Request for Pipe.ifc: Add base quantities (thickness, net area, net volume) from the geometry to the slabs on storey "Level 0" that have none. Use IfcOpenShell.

First a look at what the model holds.

```python
import ifcopenshell
import ifcopenshell.util.element
import ifcopenshell.util.unit

model = ifcopenshell.open("Pipe.ifc")
print(model.schema)
for unit_type in ("LENGTHUNIT", "AREAUNIT", "VOLUMEUNIT"):
    print(unit_type, ifcopenshell.util.unit.calculate_unit_scale(model, unit_type))
storey = next(s for s in model.by_type("IfcBuildingStorey") if s.Name == "Level 0")
slabs = [e for e in ifcopenshell.util.element.get_decomposition(storey) if e.is_a("IfcSlab")]
for e in sorted(slabs, key=lambda e: e.id()):
    print(e.id(), e.is_a(), e.Name, list(ifcopenshell.util.element.get_psets(e, qtos_only=True)), sep=" | ")
```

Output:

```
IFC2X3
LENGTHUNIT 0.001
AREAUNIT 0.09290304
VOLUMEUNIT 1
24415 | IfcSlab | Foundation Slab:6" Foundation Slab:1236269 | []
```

```python
import ifcopenshell
import ifcopenshell.api.pset
import ifcopenshell.geom
import ifcopenshell.util.element
import ifcopenshell.util.shape
import ifcopenshell.util.unit

model = ifcopenshell.open("Pipe.ifc")
unit_scale = ifcopenshell.util.unit.calculate_unit_scale(model)
area_scale = ifcopenshell.util.unit.calculate_unit_scale(model, "AREAUNIT")
volume_scale = ifcopenshell.util.unit.calculate_unit_scale(model, "VOLUMEUNIT")
settings = ifcopenshell.geom.settings()

storey = next(s for s in model.by_type("IfcBuildingStorey") if s.Name == "Level 0")
slabs = [e for e in ifcopenshell.util.element.get_decomposition(storey) if e.is_a("IfcSlab")]

for e in sorted(slabs, key=lambda e: e.id()):
    if ifcopenshell.util.element.get_psets(e, qtos_only=True, should_inherit=False):
        continue
    # Geometry comes back in metres, in the element's own axes.
    shape = ifcopenshell.geom.create_shape(settings, e)
    values = {
        "Width": ifcopenshell.util.shape.get_z(shape.geometry) / unit_scale,
        "NetArea": ifcopenshell.util.shape.get_footprint_area(shape.geometry) / area_scale,
        "NetVolume": ifcopenshell.util.shape.get_volume(shape.geometry) / volume_scale,
    }
    qto = ifcopenshell.api.pset.add_qto(model, product=e, name="BaseQuantities")
    ifcopenshell.api.pset.edit_qto(model, qto=qto, properties=values)
    print(e.id(), {k: round(v, 3) for k, v in values.items()})

model.write("Pipe_edited.ifc")
```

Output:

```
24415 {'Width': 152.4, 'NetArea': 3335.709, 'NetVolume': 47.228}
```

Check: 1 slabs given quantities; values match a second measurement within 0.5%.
